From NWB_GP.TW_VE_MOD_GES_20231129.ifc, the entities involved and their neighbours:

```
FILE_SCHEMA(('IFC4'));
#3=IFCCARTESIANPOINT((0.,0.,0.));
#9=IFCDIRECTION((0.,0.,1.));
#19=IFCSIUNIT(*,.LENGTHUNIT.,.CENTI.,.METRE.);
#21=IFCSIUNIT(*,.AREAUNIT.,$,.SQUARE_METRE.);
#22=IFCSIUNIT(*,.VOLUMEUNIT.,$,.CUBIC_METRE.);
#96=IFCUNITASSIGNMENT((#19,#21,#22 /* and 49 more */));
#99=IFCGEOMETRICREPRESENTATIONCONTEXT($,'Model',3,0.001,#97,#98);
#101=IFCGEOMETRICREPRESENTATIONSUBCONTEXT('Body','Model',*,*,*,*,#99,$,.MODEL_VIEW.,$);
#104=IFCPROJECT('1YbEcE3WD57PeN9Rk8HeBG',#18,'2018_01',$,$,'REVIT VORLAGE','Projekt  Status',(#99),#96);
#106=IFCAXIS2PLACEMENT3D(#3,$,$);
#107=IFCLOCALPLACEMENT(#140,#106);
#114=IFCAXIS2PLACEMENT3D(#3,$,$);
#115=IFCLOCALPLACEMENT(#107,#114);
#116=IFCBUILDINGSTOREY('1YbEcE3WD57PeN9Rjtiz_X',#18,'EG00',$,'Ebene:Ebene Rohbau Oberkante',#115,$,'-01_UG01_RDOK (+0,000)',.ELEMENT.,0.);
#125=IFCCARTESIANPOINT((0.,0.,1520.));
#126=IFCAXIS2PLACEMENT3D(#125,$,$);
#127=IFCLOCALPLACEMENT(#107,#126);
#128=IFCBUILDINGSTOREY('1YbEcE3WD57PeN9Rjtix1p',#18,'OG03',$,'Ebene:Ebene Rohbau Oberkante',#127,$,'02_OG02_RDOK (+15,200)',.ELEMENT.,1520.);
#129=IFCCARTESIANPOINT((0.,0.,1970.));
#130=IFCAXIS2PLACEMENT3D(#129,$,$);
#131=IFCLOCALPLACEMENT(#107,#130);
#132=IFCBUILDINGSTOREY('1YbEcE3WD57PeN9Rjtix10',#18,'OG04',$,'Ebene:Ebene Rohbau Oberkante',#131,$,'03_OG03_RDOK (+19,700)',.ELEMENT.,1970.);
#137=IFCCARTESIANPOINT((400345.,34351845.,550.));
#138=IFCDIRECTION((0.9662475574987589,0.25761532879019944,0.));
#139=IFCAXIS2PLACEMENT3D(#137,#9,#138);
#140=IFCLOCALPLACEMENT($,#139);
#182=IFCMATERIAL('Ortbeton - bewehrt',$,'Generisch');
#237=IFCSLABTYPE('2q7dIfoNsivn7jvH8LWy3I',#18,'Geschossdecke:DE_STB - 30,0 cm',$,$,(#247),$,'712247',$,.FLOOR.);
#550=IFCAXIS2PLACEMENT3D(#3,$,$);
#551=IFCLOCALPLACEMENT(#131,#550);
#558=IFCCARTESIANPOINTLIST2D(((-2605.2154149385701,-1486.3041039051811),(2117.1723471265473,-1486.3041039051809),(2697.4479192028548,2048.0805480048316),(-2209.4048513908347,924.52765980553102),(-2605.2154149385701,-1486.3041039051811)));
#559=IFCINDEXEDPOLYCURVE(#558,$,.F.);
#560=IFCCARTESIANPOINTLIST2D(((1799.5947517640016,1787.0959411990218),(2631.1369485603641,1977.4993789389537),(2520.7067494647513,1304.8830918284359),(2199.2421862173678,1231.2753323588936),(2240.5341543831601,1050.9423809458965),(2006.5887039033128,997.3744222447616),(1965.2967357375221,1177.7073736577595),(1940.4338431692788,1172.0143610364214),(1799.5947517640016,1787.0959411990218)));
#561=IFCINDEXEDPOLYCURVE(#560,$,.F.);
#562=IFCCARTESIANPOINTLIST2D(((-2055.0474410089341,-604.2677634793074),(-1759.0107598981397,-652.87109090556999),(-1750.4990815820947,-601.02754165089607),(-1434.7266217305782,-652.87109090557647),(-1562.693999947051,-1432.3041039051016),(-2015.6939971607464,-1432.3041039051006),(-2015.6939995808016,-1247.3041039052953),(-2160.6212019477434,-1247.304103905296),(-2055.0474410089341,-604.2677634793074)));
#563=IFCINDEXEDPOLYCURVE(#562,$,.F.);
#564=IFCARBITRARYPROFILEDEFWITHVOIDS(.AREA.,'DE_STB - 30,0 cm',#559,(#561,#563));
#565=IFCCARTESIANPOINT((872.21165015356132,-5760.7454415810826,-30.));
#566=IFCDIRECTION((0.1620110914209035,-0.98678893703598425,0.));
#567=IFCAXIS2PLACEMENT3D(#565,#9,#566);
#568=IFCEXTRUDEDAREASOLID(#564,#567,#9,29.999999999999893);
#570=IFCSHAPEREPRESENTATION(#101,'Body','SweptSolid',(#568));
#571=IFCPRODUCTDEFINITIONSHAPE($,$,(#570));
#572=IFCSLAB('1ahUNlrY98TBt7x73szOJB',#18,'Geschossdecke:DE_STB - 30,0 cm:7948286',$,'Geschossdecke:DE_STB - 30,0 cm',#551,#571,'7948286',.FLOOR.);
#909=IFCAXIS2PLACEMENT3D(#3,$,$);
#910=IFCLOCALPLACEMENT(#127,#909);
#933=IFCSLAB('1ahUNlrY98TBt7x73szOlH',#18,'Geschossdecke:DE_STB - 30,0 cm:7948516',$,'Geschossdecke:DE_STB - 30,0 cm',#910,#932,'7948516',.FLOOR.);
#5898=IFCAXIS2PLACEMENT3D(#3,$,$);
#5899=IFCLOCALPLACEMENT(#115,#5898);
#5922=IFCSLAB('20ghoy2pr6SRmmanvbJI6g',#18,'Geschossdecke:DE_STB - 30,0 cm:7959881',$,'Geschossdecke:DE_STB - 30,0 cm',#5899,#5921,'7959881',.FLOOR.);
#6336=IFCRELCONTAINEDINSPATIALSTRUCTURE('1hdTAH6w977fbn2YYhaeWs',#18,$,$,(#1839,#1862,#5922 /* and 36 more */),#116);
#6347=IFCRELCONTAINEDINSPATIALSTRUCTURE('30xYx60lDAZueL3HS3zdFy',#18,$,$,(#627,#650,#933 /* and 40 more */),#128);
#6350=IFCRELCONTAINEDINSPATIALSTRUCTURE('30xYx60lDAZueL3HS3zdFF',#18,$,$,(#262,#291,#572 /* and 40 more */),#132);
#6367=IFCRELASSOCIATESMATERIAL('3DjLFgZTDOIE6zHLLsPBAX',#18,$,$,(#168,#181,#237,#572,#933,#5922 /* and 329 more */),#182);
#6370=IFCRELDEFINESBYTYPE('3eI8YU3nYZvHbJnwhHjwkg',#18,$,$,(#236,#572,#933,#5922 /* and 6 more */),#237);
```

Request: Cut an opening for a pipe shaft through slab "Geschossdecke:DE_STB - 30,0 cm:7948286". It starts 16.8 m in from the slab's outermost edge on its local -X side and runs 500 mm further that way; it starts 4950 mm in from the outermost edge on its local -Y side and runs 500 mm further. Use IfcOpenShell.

```python
import numpy as np
import ifcopenshell
import ifcopenshell.api.feature
import ifcopenshell.api.geometry
import ifcopenshell.api.root
import ifcopenshell.geom
import ifcopenshell.util.placement
import ifcopenshell.util.representation
import ifcopenshell.util.shape
import ifcopenshell.util.unit

model = ifcopenshell.open("NWB_GP.TW_VE_MOD_GES_20231129.ifc")
unit_scale = ifcopenshell.util.unit.calculate_unit_scale(model)
settings = ifcopenshell.geom.settings()


def volume(element):
    """Net volume in cubic metres, openings subtracted."""
    shape = ifcopenshell.geom.create_shape(settings, element)
    return ifcopenshell.util.shape.get_volume(shape.geometry)


slab = model.by_id(572)
before = volume(slab)

# Extent in the slab's own axes, in metres. The edges named are its -X and -Y sides.
slab_shape = ifcopenshell.geom.create_shape(settings, slab)
vertices = ifcopenshell.util.shape.get_vertices(slab_shape.geometry)
x_min, y_min, bottom = vertices.min(axis=0)
top = vertices[:, 2].max()

opening = ifcopenshell.api.root.create_entity(model, ifc_class="IfcOpeningElement", name="Pipe shaft opening", predefined_type="OPENING")
context = ifcopenshell.util.representation.get_context(model, "Model", "Body", "MODEL_VIEW")
width, depth = 0.5, 0.5
outline = [(0.0, 0.0), (width, 0.0), (width, depth), (0.0, depth), (0.0, 0.0)]
# Overshoot both faces by 50 mm so the cut is clean.
shape = ifcopenshell.api.geometry.add_slab_representation(
    model, context=context, depth=top - bottom + 0.1, polyline=outline
)
ifcopenshell.api.geometry.assign_representation(model, product=opening, representation=shape)

matrix = ifcopenshell.util.placement.get_local_placement(slab.ObjectPlacement)
matrix[:, 3] = matrix @ np.append(np.array([x_min + 16.8, y_min + 4.95, bottom - 0.05]) / unit_scale, 1.0)
ifcopenshell.api.geometry.edit_object_placement(model, product=opening, matrix=matrix, is_si=False)
ifcopenshell.api.feature.add_feature(model, feature=opening, element=slab)

after = volume(slab)

print(f"slab volume {before:.3f} -> {after:.3f} m3")

model.write("NWB_GP.TW_VE_MOD_GES_20231129_edited.ifc")
```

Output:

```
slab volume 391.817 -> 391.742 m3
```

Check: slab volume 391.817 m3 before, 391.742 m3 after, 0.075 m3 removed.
